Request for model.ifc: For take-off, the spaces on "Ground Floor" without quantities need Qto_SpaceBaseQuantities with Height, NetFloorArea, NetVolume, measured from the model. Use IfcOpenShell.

First a look at what the model holds.

```python
import ifcopenshell
import ifcopenshell.util.element
import ifcopenshell.util.unit

model = ifcopenshell.open("model.ifc")
print(model.schema)
for unit_type in ("LENGTHUNIT", "AREAUNIT", "VOLUMEUNIT"):
    print(unit_type, ifcopenshell.util.unit.calculate_unit_scale(model, unit_type))
storey = next(s for s in model.by_type("IfcBuildingStorey") if s.Name == "Ground Floor")
spaces = [e for e in ifcopenshell.util.element.get_decomposition(storey) if e.is_a("IfcSpace")]
for e in sorted(spaces, key=lambda e: e.id()):
    print(e.id(), e.is_a(), e.Name, list(ifcopenshell.util.element.get_psets(e, qtos_only=True)), sep=" | ")
```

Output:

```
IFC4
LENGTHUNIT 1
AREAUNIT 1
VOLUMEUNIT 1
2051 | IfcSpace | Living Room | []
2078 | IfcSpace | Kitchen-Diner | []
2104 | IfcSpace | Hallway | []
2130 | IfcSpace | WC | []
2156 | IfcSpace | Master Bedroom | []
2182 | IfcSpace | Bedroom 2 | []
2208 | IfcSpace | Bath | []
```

```python
import ifcopenshell
import ifcopenshell.api.pset
import ifcopenshell.geom
import ifcopenshell.util.element
import ifcopenshell.util.shape
import ifcopenshell.util.unit

model = ifcopenshell.open("model.ifc")
unit_scale = ifcopenshell.util.unit.calculate_unit_scale(model)
area_scale = ifcopenshell.util.unit.calculate_unit_scale(model, "AREAUNIT")
volume_scale = ifcopenshell.util.unit.calculate_unit_scale(model, "VOLUMEUNIT")
settings = ifcopenshell.geom.settings()

storey = next(s for s in model.by_type("IfcBuildingStorey") if s.Name == "Ground Floor")
spaces = [e for e in ifcopenshell.util.element.get_decomposition(storey) if e.is_a("IfcSpace")]

for e in sorted(spaces, key=lambda e: e.id()):
    if ifcopenshell.util.element.get_psets(e, qtos_only=True, should_inherit=False):
        continue
    # Geometry comes back in metres, in the element's own axes.
    shape = ifcopenshell.geom.create_shape(settings, e)
    values = {
        "Height": ifcopenshell.util.shape.get_z(shape.geometry) / unit_scale,
        "NetFloorArea": ifcopenshell.util.shape.get_footprint_area(shape.geometry) / area_scale,
        "NetVolume": ifcopenshell.util.shape.get_volume(shape.geometry) / volume_scale,
    }
    qto = ifcopenshell.api.pset.add_qto(model, product=e, name="Qto_SpaceBaseQuantities")
    ifcopenshell.api.pset.edit_qto(model, qto=qto, properties=values)
    print(e.id(), {k: round(v, 3) for k, v in values.items()})

model.write("model_rev.ifc")
```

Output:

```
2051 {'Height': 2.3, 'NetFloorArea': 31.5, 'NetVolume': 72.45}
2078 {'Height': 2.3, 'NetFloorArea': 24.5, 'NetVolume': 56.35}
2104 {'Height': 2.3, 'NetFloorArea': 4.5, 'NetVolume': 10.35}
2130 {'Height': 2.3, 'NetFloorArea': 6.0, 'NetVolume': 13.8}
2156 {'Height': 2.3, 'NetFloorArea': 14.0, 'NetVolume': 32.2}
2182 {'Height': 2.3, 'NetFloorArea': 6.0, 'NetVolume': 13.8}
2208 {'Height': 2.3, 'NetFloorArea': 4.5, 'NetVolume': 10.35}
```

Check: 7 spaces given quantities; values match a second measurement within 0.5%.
